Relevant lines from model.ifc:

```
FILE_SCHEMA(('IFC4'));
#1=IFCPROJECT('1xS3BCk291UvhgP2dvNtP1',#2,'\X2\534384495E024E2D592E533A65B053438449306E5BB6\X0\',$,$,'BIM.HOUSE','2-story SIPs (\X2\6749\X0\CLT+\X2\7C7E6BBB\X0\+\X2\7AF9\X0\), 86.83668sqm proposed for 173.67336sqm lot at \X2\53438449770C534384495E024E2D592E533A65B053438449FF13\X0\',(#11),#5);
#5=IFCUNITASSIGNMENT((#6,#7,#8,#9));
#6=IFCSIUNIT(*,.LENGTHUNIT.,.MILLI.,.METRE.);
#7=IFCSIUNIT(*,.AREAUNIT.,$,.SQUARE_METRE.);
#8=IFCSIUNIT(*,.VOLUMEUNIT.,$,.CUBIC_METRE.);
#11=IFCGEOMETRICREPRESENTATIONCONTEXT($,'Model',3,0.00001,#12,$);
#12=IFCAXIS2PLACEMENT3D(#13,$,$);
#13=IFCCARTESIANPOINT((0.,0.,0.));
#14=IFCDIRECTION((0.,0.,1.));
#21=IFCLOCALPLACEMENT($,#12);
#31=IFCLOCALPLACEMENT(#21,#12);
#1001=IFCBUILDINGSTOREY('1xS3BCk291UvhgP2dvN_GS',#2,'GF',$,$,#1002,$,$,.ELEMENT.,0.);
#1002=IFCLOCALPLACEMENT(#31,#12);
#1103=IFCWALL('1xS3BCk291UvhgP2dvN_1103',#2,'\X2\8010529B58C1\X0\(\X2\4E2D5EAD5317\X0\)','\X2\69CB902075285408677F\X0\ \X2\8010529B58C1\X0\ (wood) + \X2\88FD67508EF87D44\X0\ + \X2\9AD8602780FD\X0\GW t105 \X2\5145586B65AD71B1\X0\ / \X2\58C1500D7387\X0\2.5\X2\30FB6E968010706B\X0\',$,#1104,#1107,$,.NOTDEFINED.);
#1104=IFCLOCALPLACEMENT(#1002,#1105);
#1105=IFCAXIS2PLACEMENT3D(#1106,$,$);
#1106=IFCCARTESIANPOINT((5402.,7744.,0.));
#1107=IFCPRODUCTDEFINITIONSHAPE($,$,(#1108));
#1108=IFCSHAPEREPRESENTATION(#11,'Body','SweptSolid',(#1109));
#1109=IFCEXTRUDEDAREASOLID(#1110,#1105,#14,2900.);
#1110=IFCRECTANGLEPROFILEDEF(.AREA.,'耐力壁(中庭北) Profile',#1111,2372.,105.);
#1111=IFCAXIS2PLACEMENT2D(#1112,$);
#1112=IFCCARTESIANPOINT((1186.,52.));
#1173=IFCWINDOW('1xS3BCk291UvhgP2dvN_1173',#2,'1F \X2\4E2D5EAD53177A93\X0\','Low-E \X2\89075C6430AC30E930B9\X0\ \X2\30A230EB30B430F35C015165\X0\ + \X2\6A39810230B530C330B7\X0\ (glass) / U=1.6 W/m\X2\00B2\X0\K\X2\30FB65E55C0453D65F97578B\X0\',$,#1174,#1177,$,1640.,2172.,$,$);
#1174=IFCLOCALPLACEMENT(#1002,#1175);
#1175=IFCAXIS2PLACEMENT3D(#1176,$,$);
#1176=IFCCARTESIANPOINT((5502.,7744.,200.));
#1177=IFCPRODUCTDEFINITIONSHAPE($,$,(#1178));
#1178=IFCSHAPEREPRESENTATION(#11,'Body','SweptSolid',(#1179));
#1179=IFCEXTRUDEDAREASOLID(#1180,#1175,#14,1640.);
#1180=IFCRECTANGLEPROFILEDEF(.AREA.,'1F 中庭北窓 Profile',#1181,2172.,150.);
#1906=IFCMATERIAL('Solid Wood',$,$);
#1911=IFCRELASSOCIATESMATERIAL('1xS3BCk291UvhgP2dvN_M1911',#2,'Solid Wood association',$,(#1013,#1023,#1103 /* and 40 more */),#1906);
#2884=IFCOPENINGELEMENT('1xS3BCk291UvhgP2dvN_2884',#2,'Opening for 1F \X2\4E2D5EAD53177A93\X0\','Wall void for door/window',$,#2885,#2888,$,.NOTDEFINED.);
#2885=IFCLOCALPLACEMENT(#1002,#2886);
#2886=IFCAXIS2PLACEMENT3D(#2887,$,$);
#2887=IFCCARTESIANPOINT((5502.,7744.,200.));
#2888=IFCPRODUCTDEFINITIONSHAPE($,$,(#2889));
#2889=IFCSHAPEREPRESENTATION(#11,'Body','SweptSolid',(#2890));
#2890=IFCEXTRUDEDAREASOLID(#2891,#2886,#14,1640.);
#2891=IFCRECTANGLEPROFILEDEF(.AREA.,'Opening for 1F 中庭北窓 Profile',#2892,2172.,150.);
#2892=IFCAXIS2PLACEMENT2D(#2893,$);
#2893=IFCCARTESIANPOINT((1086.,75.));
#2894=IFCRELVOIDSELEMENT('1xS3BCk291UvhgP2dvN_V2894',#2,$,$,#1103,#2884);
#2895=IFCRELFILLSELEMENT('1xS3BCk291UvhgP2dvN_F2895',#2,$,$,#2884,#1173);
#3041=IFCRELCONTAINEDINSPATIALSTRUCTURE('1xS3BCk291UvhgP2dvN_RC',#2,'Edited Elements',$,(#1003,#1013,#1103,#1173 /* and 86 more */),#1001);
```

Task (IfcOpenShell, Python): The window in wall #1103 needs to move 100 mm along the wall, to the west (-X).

```python
import ifcopenshell
import ifcopenshell.api.geometry
import ifcopenshell.util.placement

model = ifcopenshell.open("model.ifc")

window = model.by_id(1173)
opening = window.FillsVoids[0].RelatingOpeningElement
wall = opening.VoidsElements[0].RelatingBuildingElement

wall_matrix = ifcopenshell.util.placement.get_local_placement(wall.ObjectPlacement)
shift = wall_matrix[:3, 0] * -100.0
before = ifcopenshell.util.placement.get_local_placement(window.ObjectPlacement)[:3, 3].copy()

# The window is not placed relative to its opening, so move both.
for product in (opening, window):
    matrix = ifcopenshell.util.placement.get_local_placement(product.ObjectPlacement)
    matrix[:3, 3] += shift
    ifcopenshell.api.geometry.edit_object_placement(model, product=product, matrix=matrix, is_si=False)

after = ifcopenshell.util.placement.get_local_placement(window.ObjectPlacement)[:3, 3]
print("window moved by", (after - before).round(3) + 0.0)

model.write("model_edited.ifc")
```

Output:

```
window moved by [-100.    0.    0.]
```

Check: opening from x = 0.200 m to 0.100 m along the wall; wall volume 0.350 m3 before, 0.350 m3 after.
